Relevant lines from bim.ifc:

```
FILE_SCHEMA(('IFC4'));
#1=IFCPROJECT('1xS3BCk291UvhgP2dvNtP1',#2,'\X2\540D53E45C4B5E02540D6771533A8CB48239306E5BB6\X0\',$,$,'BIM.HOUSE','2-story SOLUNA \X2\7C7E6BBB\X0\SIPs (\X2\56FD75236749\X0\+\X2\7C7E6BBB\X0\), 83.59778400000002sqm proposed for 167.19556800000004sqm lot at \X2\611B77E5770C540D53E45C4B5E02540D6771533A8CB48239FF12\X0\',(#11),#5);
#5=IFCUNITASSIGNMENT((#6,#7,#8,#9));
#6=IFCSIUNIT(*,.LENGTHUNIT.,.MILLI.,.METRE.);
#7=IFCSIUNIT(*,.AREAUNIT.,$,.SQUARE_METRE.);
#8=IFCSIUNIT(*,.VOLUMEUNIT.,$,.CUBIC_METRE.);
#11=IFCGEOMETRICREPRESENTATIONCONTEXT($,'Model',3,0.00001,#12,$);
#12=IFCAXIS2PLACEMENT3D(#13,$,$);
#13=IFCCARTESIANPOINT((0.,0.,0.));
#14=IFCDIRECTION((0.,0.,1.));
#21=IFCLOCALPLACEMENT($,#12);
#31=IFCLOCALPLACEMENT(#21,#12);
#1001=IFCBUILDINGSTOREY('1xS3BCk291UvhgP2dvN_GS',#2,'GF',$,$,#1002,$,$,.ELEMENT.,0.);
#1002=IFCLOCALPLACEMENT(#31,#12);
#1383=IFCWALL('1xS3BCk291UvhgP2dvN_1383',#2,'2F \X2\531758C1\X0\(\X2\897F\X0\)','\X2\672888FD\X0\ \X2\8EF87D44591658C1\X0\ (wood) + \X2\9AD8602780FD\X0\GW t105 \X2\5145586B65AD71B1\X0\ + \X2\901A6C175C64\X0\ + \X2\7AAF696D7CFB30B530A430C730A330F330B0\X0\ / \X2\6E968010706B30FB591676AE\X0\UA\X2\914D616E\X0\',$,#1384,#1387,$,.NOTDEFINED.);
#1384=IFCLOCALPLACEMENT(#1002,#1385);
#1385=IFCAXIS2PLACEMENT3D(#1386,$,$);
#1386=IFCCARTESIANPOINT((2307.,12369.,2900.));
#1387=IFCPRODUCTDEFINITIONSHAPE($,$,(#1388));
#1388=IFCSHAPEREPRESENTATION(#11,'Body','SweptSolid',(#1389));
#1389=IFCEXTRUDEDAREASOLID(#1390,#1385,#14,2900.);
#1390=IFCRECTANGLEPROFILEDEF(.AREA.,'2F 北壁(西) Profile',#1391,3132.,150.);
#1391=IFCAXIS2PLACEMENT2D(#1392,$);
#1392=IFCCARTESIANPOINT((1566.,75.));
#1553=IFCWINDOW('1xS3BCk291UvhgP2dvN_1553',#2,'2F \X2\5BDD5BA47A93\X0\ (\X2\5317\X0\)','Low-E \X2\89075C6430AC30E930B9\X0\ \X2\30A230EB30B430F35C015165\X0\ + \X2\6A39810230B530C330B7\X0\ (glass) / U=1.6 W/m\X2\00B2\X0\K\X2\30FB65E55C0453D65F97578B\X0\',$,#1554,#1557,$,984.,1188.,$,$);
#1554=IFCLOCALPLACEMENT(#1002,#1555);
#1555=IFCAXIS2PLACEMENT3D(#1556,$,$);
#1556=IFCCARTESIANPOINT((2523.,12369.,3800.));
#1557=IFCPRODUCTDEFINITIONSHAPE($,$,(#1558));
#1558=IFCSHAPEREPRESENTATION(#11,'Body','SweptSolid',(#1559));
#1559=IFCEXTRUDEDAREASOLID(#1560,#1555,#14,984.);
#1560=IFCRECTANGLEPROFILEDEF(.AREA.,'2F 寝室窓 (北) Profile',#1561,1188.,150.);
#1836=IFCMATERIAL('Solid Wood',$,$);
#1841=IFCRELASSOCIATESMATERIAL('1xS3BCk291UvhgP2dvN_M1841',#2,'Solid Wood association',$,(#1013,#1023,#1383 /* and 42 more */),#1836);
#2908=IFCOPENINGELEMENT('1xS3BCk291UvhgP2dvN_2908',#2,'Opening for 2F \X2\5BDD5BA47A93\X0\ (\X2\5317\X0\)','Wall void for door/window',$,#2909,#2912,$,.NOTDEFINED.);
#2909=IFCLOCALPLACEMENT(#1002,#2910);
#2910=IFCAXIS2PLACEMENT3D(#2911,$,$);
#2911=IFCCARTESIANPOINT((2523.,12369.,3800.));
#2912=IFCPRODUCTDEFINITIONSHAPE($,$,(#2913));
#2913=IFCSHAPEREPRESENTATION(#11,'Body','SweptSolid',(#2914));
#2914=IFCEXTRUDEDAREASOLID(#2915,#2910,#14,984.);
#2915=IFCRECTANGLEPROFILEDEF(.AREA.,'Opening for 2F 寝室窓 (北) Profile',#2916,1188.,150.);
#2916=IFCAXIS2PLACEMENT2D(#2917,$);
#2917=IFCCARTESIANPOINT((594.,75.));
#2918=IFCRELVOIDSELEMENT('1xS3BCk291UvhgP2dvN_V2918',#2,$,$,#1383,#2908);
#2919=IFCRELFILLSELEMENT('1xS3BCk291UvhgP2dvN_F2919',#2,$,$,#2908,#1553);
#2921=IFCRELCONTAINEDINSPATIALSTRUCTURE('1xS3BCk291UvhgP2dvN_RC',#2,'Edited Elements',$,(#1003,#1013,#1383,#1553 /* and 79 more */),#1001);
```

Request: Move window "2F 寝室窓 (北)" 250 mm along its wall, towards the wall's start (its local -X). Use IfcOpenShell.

```python
import ifcopenshell
import ifcopenshell.api.geometry
import ifcopenshell.util.placement

model = ifcopenshell.open("bim.ifc")

window = model.by_guid("1xS3BCk291UvhgP2dvN_1553")
opening = window.FillsVoids[0].RelatingOpeningElement
wall = opening.VoidsElements[0].RelatingBuildingElement

wall_matrix = ifcopenshell.util.placement.get_local_placement(wall.ObjectPlacement)
shift = wall_matrix[:3, 0] * -250.0
before = ifcopenshell.util.placement.get_local_placement(window.ObjectPlacement)[:3, 3].copy()

# The window is not placed relative to its opening, so move both.
for product in (opening, window):
    matrix = ifcopenshell.util.placement.get_local_placement(product.ObjectPlacement)
    matrix[:3, 3] += shift
    ifcopenshell.api.geometry.edit_object_placement(model, product=product, matrix=matrix, is_si=False)

after = ifcopenshell.util.placement.get_local_placement(window.ObjectPlacement)[:3, 3]
print("window moved by", (after - before).round(3) + 0.0)

model.write("bim-out.ifc")
```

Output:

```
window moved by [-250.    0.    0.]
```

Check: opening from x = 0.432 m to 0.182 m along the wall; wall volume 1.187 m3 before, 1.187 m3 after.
